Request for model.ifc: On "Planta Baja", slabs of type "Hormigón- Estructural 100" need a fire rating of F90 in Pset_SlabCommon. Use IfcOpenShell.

First a look at what the model holds.

```python
import ifcopenshell
import ifcopenshell.util.element

model = ifcopenshell.open("model.ifc")
print(model.schema)
storey = next(s for s in model.by_type("IfcBuildingStorey") if s.Name == "Planta Baja")
slabs = [e for e in ifcopenshell.util.element.get_decomposition(storey) if e.is_a("IfcSlab")]
seen = {}
for e in slabs:
    element_type = ifcopenshell.util.element.get_type(e)
    key = (element_type.Name if element_type != e and element_type else None, ifcopenshell.util.element.get_pset(e, "Pset_SlabCommon", "FireRating"))
    seen[key] = seen.get(key, 0) + 1
for (name, value), count in sorted(seen.items(), key=str):
    print(count, "x", name, "|", value)
```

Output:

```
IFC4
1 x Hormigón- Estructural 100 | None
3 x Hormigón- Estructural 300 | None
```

```python
import ifcopenshell
import ifcopenshell.api.pset
import ifcopenshell.util.element

model = ifcopenshell.open("model.ifc")

storey = next(s for s in model.by_type("IfcBuildingStorey") if s.Name == "Planta Baja")
slabs = [e for e in ifcopenshell.util.element.get_decomposition(storey) if e.is_a("IfcSlab")]

count = 0
for e in slabs:
    element_type = ifcopenshell.util.element.get_type(e)
    if element_type in (None, e) or element_type.Name != "Hormigón- Estructural 100":
        continue
    # add_pset returns the element's existing set when there is one.
    pset = ifcopenshell.api.pset.add_pset(model, product=e, name="Pset_SlabCommon")
    ifcopenshell.api.pset.edit_pset(model, pset=pset, properties={"FireRating": "F90"})
    count += 1

print(count, "slabs updated")

model.write("model_rev.ifc")
```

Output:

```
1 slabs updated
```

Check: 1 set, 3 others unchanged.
